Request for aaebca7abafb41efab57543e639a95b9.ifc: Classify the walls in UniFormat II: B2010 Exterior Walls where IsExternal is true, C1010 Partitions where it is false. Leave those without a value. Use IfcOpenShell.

First a look at what the model holds.

```python
import ifcopenshell
import ifcopenshell.util.element

model = ifcopenshell.open("aaebca7abafb41efab57543e639a95b9.ifc")
print(model.schema)
print("classifications:", [c.Name for c in model.by_type("IfcClassification")])
values = [ifcopenshell.util.element.get_pset(e, "Pset_WallCommon", "IsExternal") for e in model.by_type("IfcWall")]
for value in (True, False, None):
    print("IsExternal", value, values.count(value))
```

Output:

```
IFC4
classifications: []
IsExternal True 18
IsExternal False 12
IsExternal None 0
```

```python
import ifcopenshell
import ifcopenshell.api.classification
import ifcopenshell.util.element

model = ifcopenshell.open("aaebca7abafb41efab57543e639a95b9.ifc")

system = ifcopenshell.api.classification.add_classification(model, classification="UniFormat II")

walls = model.by_type("IfcWall")
external = {e: ifcopenshell.util.element.get_pset(e, "Pset_WallCommon", "IsExternal") for e in walls}
for flag, code, name in ((True, "B2010", "Exterior Walls"), (False, "C1010", "Partitions")):
    products = [e for e in walls if external[e] is flag]
    ifcopenshell.api.classification.add_reference(
        model, products=products, classification=system, identification=code, name=name
    )
    print(code, len(products))

model.write("aaebca7abafb41efab57543e639a95b9_updated.ifc")
```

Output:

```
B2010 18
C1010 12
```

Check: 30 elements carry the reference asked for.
